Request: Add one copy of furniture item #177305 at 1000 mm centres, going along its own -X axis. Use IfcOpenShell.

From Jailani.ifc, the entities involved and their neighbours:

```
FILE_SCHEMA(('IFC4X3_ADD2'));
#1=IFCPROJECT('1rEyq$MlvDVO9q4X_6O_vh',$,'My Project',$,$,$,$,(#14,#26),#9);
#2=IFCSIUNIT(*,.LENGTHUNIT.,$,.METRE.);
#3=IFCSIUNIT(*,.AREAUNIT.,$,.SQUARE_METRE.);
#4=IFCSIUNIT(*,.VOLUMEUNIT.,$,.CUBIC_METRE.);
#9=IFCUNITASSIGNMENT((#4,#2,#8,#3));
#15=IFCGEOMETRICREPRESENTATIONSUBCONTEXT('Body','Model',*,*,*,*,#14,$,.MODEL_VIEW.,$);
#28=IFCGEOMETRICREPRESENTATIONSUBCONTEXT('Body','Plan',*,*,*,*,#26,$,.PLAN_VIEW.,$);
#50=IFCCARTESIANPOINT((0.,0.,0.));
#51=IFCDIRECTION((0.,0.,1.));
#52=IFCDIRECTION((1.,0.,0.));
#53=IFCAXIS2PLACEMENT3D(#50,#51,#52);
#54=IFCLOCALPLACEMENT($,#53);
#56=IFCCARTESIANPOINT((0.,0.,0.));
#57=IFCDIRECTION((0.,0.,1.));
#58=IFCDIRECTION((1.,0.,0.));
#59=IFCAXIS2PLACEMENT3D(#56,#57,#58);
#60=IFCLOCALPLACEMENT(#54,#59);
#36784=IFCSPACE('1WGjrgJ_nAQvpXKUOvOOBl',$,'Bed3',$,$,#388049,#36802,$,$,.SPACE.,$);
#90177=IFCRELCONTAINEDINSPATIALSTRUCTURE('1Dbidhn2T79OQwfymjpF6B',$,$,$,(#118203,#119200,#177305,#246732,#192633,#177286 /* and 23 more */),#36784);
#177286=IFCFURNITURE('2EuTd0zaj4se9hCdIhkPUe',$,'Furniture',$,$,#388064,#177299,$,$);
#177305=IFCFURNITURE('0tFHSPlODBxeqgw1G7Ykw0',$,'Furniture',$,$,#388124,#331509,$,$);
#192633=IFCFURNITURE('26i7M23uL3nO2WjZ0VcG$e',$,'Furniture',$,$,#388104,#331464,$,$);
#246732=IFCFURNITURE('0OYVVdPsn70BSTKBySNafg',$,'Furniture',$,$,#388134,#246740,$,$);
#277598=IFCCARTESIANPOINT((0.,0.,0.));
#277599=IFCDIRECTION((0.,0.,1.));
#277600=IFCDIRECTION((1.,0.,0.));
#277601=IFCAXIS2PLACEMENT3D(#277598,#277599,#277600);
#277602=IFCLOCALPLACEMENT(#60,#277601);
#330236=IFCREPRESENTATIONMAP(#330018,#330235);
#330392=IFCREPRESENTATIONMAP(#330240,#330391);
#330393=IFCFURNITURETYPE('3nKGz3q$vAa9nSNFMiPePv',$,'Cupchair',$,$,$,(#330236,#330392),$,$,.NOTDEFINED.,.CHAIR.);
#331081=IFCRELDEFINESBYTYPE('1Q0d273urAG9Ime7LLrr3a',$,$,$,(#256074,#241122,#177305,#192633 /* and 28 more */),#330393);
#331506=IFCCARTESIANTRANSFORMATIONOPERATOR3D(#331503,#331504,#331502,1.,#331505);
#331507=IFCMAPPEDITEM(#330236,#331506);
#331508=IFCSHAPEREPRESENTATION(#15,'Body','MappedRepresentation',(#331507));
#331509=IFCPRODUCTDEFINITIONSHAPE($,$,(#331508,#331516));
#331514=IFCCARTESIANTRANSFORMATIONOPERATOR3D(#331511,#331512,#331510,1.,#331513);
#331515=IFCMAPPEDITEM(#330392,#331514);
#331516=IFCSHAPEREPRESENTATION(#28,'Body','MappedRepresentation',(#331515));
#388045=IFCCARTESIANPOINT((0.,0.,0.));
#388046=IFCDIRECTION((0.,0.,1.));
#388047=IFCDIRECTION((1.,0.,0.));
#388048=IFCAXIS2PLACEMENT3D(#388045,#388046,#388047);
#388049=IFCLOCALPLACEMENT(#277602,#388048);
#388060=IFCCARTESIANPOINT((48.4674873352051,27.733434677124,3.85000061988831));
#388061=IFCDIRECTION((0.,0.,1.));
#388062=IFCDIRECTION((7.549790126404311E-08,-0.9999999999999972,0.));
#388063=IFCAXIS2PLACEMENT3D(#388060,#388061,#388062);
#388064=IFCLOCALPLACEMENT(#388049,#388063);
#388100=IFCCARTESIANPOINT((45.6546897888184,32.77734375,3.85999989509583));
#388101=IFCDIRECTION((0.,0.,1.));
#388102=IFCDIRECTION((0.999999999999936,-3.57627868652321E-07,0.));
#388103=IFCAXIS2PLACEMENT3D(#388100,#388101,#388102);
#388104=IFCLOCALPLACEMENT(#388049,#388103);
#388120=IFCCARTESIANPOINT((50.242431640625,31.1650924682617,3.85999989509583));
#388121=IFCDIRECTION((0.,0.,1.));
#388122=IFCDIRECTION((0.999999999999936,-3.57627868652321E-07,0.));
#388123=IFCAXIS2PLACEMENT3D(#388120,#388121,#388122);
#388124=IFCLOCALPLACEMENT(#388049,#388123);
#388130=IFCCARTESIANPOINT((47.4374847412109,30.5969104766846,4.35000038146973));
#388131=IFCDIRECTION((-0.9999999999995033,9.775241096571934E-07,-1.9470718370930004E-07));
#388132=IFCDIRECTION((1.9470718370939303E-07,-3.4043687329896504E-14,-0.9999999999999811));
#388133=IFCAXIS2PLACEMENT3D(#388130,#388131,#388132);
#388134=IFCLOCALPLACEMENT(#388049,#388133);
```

```python
import ifcopenshell
import ifcopenshell.api.geometry
import ifcopenshell.api.root
import ifcopenshell.util.element
import ifcopenshell.util.placement
import ifcopenshell.util.unit

model = ifcopenshell.open("Jailani.ifc")
unit_scale = ifcopenshell.util.unit.calculate_unit_scale(model)

source = model.by_guid("0tFHSPlODBxeqgw1G7Ykw0")
base = ifcopenshell.util.placement.get_local_placement(source.ObjectPlacement)
step = -base[:3, 0] * 1 / unit_scale

for i in range(1, 2):
    copy = ifcopenshell.api.root.copy_class(model, product=source)
    copy.Representation = ifcopenshell.util.element.copy_deep(
        model, source.Representation, exclude=["IfcGeometricRepresentationContext", "IfcRepresentationMap"]
    )
    matrix = base.copy()
    matrix[:3, 3] += i * step
    print("added at", matrix[:3, 3].round(3) + 0.0)
    ifcopenshell.api.geometry.edit_object_placement(model, product=copy, matrix=matrix, is_si=False)

model.write("Jailani_edited.ifc")
```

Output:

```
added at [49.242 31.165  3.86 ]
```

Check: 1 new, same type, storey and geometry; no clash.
